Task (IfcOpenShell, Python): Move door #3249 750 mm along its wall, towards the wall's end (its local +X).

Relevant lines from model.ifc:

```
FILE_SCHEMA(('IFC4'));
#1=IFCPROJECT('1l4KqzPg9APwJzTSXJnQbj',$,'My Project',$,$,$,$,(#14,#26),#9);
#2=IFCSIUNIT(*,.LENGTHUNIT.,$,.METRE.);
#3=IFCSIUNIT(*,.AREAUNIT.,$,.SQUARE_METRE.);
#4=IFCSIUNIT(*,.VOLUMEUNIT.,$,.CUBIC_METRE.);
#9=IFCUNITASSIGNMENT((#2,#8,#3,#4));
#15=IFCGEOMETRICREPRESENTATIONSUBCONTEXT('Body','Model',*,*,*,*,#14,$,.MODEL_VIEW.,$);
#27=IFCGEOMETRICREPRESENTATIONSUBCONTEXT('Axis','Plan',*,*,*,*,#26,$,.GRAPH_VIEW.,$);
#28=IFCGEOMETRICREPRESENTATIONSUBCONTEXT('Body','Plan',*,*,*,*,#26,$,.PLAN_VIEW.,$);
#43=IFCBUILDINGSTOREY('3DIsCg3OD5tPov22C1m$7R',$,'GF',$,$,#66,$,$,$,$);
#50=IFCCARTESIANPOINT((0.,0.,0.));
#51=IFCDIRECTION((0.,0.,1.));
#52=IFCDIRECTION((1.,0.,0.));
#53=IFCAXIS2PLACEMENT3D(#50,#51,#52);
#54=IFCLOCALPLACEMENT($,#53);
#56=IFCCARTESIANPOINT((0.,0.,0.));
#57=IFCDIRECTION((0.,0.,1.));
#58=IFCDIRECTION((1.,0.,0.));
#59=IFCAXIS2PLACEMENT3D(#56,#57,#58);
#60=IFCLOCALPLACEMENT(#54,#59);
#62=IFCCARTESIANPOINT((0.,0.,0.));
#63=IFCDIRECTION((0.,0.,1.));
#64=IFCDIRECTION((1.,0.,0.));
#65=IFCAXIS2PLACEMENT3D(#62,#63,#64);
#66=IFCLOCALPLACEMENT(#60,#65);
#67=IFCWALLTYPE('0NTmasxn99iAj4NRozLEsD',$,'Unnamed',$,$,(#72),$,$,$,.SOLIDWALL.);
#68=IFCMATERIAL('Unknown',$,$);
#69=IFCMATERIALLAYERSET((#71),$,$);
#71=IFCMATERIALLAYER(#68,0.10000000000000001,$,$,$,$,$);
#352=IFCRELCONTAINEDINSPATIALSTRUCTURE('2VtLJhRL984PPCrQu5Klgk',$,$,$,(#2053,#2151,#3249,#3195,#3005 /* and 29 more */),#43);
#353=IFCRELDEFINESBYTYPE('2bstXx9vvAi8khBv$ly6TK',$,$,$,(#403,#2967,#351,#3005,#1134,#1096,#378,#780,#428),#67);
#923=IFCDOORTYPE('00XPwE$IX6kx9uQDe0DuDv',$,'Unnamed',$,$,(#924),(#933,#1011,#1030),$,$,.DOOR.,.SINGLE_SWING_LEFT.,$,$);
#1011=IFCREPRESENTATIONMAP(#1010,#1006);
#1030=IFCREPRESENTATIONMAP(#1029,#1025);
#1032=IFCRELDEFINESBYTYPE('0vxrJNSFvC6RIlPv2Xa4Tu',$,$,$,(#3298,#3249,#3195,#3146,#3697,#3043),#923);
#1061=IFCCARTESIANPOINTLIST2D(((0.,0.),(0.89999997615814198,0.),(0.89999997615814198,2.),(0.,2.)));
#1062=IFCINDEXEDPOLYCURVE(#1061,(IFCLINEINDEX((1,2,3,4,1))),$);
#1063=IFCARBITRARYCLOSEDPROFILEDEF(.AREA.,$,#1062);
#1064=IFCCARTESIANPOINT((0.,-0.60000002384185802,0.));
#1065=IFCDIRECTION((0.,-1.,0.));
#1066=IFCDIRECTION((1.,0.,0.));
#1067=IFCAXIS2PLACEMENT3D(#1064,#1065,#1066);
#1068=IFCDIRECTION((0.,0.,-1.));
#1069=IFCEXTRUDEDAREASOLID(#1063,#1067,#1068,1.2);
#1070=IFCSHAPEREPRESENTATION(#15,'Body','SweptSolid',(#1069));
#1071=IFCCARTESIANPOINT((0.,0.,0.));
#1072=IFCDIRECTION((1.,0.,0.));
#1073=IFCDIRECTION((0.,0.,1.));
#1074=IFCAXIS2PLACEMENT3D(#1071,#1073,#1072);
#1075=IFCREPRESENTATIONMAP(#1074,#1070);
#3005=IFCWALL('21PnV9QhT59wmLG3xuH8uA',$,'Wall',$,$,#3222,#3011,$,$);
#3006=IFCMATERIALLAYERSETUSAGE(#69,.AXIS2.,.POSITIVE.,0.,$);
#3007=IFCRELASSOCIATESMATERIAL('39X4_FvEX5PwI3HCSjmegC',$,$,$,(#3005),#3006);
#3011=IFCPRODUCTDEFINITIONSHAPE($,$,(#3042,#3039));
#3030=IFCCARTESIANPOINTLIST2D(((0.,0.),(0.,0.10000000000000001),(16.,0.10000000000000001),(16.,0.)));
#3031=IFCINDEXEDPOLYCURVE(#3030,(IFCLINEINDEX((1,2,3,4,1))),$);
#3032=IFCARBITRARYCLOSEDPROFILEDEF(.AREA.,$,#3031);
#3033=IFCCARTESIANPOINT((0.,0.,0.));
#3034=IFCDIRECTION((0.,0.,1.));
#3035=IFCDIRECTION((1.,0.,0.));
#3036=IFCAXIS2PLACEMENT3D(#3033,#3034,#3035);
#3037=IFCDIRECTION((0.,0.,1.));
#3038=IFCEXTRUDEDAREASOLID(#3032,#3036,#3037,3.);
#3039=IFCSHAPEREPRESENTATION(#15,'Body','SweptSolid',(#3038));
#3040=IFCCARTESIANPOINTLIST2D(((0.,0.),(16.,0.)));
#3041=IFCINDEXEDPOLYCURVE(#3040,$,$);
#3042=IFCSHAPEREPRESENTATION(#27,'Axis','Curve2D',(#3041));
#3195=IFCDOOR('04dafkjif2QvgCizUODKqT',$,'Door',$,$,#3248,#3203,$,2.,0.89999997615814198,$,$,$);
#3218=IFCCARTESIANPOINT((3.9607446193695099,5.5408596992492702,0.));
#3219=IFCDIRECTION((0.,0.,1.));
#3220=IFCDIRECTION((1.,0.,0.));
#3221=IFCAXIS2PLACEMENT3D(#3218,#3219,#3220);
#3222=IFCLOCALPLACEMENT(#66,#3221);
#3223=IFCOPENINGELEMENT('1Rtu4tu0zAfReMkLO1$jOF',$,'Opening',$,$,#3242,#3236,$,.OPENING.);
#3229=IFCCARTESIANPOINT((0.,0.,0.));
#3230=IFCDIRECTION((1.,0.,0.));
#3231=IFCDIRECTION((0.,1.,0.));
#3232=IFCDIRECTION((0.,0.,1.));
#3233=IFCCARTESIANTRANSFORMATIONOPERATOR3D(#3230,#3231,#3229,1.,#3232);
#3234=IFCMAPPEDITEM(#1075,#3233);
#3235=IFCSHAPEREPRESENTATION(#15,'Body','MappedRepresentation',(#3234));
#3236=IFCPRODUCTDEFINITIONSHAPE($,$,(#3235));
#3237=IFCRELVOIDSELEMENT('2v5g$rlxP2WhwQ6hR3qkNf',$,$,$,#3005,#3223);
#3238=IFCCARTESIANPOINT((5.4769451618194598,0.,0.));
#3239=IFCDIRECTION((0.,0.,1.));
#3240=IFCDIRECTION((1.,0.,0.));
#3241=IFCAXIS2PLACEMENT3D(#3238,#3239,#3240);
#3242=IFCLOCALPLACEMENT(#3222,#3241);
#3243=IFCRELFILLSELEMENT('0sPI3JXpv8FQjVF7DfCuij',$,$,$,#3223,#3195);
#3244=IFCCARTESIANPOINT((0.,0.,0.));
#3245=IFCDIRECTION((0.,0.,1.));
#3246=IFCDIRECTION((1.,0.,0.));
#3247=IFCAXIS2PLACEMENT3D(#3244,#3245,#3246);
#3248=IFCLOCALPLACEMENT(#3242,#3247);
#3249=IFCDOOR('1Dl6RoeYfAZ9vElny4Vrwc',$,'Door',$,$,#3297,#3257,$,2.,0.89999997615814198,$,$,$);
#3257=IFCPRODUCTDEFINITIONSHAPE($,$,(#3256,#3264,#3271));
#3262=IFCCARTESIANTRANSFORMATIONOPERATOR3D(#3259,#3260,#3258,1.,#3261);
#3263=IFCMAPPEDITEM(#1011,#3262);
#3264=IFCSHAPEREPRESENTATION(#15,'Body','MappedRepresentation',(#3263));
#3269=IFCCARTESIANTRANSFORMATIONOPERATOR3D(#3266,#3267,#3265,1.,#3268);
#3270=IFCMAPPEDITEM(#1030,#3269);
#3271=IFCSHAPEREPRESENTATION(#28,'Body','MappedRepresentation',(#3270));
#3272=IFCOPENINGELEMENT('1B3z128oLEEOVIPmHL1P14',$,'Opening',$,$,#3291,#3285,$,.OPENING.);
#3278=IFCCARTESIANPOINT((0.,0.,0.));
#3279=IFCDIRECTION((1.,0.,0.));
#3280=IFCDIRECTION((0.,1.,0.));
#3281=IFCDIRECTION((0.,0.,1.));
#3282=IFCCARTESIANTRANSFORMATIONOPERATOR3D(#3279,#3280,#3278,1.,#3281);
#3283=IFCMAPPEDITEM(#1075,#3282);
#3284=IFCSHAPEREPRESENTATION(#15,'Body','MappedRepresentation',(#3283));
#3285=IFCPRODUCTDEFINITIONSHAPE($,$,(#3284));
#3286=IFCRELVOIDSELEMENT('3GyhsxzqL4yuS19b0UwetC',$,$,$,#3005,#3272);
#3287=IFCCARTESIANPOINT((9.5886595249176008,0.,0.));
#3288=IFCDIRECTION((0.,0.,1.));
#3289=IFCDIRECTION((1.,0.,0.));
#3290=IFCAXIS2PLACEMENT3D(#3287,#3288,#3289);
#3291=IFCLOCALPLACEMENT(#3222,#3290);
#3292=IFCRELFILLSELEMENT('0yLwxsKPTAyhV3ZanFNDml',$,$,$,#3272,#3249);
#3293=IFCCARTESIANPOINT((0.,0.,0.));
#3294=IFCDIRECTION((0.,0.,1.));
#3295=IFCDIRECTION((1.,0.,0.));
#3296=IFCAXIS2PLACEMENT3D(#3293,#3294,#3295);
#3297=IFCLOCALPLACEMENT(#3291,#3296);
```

```python
import ifcopenshell
import ifcopenshell.api.geometry
import ifcopenshell.util.placement

model = ifcopenshell.open("model.ifc")

door = model.by_guid("1Dl6RoeYfAZ9vElny4Vrwc")
opening = door.FillsVoids[0].RelatingOpeningElement
wall = opening.VoidsElements[0].RelatingBuildingElement

wall_matrix = ifcopenshell.util.placement.get_local_placement(wall.ObjectPlacement)
shift = wall_matrix[:3, 0] * 0.75
before = ifcopenshell.util.placement.get_local_placement(door.ObjectPlacement)[:3, 3].copy()

# The door is placed relative to its opening, so it follows when the opening moves.
matrix = ifcopenshell.util.placement.get_local_placement(opening.ObjectPlacement)
matrix[:3, 3] += shift
ifcopenshell.api.geometry.edit_object_placement(
    model, product=opening, matrix=matrix, is_si=False, should_transform_children=True
)

after = ifcopenshell.util.placement.get_local_placement(door.ObjectPlacement)[:3, 3]
print("door moved by", (after - before).round(3) + 0.0)

model.write("model_rev.ifc")
```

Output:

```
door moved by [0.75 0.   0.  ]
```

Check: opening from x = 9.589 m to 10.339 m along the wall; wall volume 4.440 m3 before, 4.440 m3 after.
